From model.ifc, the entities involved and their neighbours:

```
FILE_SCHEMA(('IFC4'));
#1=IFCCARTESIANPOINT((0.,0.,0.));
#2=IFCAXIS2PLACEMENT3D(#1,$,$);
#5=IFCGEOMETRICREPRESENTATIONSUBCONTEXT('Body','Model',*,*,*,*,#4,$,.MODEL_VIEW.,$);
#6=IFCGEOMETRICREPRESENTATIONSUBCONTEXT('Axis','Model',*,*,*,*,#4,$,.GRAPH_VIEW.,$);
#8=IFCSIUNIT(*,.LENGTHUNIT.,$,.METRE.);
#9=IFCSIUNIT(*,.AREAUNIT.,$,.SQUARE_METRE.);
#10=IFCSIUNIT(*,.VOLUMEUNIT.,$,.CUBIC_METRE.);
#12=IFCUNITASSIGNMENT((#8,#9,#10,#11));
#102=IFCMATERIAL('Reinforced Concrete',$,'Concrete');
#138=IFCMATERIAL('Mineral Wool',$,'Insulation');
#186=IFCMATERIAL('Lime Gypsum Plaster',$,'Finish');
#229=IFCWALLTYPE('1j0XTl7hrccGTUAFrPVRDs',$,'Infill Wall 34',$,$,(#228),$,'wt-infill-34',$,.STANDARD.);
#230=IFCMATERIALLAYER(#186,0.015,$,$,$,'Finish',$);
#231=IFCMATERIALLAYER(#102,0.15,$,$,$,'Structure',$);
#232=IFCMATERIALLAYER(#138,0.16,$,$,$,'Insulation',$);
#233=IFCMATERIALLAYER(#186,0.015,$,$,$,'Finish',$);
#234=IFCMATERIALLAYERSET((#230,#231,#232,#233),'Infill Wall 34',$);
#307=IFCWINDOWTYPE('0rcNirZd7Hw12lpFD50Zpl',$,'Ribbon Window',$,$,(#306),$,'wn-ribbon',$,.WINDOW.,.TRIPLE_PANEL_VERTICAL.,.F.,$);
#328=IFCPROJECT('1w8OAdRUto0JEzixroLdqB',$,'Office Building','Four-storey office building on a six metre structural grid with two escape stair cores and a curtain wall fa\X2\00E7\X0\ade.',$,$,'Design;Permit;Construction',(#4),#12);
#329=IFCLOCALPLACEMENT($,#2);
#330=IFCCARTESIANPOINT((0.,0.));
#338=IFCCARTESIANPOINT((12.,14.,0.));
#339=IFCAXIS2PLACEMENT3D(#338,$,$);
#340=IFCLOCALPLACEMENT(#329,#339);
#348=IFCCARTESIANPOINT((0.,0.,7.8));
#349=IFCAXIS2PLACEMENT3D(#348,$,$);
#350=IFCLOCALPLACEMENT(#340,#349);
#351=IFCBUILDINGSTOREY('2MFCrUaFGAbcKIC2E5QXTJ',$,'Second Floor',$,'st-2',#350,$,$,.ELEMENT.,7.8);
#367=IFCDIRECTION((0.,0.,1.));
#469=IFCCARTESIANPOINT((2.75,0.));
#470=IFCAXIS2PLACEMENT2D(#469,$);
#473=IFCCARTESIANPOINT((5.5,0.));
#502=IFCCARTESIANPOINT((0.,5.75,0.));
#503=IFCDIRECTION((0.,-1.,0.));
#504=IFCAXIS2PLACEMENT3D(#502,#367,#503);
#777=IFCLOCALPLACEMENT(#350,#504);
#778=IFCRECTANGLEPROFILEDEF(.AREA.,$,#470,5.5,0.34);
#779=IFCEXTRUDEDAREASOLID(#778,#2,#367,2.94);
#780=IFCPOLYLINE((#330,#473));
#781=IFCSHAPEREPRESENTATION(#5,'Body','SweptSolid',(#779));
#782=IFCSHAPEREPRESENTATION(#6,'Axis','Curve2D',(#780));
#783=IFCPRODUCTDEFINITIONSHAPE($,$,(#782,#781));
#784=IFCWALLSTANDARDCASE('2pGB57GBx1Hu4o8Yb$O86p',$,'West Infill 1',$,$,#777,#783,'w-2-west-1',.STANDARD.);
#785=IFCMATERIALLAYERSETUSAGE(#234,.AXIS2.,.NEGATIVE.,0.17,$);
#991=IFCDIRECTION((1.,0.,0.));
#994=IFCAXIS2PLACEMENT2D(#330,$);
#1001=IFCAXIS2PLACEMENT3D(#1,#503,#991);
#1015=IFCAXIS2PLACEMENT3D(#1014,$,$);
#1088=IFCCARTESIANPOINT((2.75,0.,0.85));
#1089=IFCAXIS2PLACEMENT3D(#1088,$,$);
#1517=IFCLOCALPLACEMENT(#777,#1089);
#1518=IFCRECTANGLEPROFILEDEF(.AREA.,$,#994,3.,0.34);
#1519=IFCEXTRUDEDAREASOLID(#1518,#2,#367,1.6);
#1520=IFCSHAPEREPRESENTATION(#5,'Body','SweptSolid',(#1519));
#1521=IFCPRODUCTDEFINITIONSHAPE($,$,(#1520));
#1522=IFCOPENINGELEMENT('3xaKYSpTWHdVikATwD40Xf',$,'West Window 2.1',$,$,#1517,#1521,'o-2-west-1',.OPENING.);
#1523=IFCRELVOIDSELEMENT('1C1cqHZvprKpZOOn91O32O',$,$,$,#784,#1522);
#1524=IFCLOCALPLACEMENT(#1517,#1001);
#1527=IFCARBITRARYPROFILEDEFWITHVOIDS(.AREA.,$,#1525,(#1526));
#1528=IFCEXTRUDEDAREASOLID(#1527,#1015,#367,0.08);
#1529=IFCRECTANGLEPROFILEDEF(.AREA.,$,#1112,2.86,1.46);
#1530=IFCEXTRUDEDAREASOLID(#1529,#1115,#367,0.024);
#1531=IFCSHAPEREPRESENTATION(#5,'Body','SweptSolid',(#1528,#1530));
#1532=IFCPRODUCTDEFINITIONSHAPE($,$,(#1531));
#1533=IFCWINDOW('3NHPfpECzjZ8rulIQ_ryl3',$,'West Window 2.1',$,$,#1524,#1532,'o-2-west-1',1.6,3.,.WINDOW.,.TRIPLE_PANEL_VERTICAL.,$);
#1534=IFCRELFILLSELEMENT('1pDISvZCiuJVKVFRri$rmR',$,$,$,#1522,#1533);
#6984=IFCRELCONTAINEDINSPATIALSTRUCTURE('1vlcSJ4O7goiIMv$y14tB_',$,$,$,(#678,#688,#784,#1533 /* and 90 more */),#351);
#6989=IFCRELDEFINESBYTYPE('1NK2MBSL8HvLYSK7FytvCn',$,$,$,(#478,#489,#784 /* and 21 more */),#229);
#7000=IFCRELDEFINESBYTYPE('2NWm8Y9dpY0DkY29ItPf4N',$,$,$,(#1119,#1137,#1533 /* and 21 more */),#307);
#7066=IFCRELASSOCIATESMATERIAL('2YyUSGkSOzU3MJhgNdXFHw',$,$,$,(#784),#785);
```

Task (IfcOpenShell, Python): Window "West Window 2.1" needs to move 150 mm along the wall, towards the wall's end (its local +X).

```python
import ifcopenshell
import ifcopenshell.api.geometry
import ifcopenshell.util.placement
import ifcopenshell.util.unit

model = ifcopenshell.open("model.ifc")
unit_scale = ifcopenshell.util.unit.calculate_unit_scale(model)

window = model.by_guid("3NHPfpECzjZ8rulIQ_ryl3")
opening = window.FillsVoids[0].RelatingOpeningElement
wall = opening.VoidsElements[0].RelatingBuildingElement

wall_matrix = ifcopenshell.util.placement.get_local_placement(wall.ObjectPlacement)
shift = wall_matrix[:3, 0] * 0.15 / unit_scale
before = ifcopenshell.util.placement.get_local_placement(window.ObjectPlacement)[:3, 3].copy()

# The window is placed relative to its opening, so it follows when the opening moves.
matrix = ifcopenshell.util.placement.get_local_placement(opening.ObjectPlacement)
matrix[:3, 3] += shift
ifcopenshell.api.geometry.edit_object_placement(
    model, product=opening, matrix=matrix, is_si=False, should_transform_children=True
)

after = ifcopenshell.util.placement.get_local_placement(window.ObjectPlacement)[:3, 3]
print("window moved by", (after - before).round(3) + 0.0)

model.write("model_updated.ifc")
```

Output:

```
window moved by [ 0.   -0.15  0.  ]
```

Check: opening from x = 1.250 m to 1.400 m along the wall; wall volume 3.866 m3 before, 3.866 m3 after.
